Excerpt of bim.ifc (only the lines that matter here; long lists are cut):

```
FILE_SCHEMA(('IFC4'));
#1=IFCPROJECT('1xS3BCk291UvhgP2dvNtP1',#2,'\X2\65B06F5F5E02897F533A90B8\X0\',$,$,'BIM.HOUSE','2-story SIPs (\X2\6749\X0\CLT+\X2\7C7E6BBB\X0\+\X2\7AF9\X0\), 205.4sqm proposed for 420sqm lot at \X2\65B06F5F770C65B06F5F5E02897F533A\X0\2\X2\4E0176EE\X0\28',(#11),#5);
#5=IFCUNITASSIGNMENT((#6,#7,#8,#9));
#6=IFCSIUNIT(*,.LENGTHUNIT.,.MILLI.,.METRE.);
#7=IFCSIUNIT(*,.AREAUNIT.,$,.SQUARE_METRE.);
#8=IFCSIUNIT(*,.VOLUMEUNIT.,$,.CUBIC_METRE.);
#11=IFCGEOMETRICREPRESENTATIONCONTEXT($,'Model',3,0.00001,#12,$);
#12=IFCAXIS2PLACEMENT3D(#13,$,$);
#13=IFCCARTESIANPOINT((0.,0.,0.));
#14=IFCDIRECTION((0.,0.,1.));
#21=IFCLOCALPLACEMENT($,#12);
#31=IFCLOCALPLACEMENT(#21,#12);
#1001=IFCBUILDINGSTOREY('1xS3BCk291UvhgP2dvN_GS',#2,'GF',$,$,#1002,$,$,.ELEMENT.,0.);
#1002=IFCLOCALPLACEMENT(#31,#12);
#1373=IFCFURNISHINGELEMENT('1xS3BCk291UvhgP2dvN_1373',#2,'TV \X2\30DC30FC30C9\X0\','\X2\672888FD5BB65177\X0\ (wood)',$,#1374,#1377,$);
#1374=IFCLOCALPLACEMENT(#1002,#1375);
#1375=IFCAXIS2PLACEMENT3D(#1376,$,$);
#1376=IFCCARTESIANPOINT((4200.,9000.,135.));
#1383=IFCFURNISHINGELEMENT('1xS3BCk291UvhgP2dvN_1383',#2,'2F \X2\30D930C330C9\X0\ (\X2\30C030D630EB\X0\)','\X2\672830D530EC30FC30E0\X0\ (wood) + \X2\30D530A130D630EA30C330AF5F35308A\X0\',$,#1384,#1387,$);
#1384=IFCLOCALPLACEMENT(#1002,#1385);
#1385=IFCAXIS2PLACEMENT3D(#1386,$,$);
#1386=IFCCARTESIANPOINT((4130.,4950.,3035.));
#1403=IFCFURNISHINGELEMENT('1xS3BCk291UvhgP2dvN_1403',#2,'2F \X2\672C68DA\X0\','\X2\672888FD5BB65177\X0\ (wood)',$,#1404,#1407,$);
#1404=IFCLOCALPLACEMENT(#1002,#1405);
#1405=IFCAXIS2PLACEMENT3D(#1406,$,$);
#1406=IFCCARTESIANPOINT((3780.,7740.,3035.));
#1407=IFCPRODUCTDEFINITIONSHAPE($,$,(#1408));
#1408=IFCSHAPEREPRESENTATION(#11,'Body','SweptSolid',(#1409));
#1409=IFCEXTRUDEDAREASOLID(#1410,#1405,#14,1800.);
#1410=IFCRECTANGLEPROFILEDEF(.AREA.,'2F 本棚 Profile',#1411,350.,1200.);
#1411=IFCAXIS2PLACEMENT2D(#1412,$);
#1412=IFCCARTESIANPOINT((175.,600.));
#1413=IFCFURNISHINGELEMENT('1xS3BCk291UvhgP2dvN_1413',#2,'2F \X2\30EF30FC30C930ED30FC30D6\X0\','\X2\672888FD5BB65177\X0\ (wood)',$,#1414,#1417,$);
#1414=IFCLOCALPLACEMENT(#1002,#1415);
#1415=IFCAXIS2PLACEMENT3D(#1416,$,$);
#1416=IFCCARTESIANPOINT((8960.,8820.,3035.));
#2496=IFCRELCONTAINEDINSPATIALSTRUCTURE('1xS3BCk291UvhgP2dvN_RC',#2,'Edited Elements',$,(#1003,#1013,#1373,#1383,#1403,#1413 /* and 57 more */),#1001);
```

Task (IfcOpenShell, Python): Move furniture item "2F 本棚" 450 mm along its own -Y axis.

```python
import ifcopenshell
import ifcopenshell.api.geometry
import ifcopenshell.util.placement

model = ifcopenshell.open("bim.ifc")

item = model.by_id(1403)
matrix = ifcopenshell.util.placement.get_local_placement(item.ObjectPlacement)
matrix[:3, 3] -= matrix[:3, 1] * 450.0
ifcopenshell.api.geometry.edit_object_placement(model, product=item, matrix=matrix, is_si=False)

print(ifcopenshell.util.placement.get_local_placement(item.ObjectPlacement).round(3) + 0.0)

model.write("bim_rev.ifc")
```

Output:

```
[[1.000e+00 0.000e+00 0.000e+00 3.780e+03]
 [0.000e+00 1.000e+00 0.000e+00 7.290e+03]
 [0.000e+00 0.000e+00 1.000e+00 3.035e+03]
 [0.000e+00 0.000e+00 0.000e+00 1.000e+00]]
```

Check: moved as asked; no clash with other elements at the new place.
